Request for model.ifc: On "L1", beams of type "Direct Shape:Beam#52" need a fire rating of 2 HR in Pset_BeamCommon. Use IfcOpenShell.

First a look at what the model holds.

```python
import ifcopenshell
import ifcopenshell.util.element

model = ifcopenshell.open("model.ifc")
print(model.schema)
storey = next(s for s in model.by_type("IfcBuildingStorey") if s.Name == "L1")
beams = [e for e in ifcopenshell.util.element.get_decomposition(storey) if e.is_a("IfcBeam")]
seen = {}
for e in beams:
    element_type = ifcopenshell.util.element.get_type(e)
    key = (element_type.Name if element_type != e and element_type else None, ifcopenshell.util.element.get_pset(e, "Pset_BeamCommon", "FireRating"))
    seen[key] = seen.get(key, 0) + 1
for (name, value), count in sorted(seen.items(), key=str):
    print(count, "x", name, "|", value)
```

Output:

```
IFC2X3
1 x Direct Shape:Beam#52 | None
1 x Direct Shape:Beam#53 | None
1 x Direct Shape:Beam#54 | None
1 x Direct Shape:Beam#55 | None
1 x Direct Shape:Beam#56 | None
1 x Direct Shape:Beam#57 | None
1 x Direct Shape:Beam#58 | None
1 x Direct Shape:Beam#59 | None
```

```python
import ifcopenshell
import ifcopenshell.api.pset
import ifcopenshell.util.element

model = ifcopenshell.open("model.ifc")

storey = next(s for s in model.by_type("IfcBuildingStorey") if s.Name == "L1")
beams = [e for e in ifcopenshell.util.element.get_decomposition(storey) if e.is_a("IfcBeam")]

count = 0
for e in beams:
    element_type = ifcopenshell.util.element.get_type(e)
    if element_type in (None, e) or element_type.Name != "Direct Shape:Beam#52":
        continue
    # add_pset returns the element's existing set when there is one.
    pset = ifcopenshell.api.pset.add_pset(model, product=e, name="Pset_BeamCommon")
    ifcopenshell.api.pset.edit_pset(model, pset=pset, properties={"FireRating": "2 HR"})
    count += 1

print(count, "beams updated")

model.write("model-out.ifc")
```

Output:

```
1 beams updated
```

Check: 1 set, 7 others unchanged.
